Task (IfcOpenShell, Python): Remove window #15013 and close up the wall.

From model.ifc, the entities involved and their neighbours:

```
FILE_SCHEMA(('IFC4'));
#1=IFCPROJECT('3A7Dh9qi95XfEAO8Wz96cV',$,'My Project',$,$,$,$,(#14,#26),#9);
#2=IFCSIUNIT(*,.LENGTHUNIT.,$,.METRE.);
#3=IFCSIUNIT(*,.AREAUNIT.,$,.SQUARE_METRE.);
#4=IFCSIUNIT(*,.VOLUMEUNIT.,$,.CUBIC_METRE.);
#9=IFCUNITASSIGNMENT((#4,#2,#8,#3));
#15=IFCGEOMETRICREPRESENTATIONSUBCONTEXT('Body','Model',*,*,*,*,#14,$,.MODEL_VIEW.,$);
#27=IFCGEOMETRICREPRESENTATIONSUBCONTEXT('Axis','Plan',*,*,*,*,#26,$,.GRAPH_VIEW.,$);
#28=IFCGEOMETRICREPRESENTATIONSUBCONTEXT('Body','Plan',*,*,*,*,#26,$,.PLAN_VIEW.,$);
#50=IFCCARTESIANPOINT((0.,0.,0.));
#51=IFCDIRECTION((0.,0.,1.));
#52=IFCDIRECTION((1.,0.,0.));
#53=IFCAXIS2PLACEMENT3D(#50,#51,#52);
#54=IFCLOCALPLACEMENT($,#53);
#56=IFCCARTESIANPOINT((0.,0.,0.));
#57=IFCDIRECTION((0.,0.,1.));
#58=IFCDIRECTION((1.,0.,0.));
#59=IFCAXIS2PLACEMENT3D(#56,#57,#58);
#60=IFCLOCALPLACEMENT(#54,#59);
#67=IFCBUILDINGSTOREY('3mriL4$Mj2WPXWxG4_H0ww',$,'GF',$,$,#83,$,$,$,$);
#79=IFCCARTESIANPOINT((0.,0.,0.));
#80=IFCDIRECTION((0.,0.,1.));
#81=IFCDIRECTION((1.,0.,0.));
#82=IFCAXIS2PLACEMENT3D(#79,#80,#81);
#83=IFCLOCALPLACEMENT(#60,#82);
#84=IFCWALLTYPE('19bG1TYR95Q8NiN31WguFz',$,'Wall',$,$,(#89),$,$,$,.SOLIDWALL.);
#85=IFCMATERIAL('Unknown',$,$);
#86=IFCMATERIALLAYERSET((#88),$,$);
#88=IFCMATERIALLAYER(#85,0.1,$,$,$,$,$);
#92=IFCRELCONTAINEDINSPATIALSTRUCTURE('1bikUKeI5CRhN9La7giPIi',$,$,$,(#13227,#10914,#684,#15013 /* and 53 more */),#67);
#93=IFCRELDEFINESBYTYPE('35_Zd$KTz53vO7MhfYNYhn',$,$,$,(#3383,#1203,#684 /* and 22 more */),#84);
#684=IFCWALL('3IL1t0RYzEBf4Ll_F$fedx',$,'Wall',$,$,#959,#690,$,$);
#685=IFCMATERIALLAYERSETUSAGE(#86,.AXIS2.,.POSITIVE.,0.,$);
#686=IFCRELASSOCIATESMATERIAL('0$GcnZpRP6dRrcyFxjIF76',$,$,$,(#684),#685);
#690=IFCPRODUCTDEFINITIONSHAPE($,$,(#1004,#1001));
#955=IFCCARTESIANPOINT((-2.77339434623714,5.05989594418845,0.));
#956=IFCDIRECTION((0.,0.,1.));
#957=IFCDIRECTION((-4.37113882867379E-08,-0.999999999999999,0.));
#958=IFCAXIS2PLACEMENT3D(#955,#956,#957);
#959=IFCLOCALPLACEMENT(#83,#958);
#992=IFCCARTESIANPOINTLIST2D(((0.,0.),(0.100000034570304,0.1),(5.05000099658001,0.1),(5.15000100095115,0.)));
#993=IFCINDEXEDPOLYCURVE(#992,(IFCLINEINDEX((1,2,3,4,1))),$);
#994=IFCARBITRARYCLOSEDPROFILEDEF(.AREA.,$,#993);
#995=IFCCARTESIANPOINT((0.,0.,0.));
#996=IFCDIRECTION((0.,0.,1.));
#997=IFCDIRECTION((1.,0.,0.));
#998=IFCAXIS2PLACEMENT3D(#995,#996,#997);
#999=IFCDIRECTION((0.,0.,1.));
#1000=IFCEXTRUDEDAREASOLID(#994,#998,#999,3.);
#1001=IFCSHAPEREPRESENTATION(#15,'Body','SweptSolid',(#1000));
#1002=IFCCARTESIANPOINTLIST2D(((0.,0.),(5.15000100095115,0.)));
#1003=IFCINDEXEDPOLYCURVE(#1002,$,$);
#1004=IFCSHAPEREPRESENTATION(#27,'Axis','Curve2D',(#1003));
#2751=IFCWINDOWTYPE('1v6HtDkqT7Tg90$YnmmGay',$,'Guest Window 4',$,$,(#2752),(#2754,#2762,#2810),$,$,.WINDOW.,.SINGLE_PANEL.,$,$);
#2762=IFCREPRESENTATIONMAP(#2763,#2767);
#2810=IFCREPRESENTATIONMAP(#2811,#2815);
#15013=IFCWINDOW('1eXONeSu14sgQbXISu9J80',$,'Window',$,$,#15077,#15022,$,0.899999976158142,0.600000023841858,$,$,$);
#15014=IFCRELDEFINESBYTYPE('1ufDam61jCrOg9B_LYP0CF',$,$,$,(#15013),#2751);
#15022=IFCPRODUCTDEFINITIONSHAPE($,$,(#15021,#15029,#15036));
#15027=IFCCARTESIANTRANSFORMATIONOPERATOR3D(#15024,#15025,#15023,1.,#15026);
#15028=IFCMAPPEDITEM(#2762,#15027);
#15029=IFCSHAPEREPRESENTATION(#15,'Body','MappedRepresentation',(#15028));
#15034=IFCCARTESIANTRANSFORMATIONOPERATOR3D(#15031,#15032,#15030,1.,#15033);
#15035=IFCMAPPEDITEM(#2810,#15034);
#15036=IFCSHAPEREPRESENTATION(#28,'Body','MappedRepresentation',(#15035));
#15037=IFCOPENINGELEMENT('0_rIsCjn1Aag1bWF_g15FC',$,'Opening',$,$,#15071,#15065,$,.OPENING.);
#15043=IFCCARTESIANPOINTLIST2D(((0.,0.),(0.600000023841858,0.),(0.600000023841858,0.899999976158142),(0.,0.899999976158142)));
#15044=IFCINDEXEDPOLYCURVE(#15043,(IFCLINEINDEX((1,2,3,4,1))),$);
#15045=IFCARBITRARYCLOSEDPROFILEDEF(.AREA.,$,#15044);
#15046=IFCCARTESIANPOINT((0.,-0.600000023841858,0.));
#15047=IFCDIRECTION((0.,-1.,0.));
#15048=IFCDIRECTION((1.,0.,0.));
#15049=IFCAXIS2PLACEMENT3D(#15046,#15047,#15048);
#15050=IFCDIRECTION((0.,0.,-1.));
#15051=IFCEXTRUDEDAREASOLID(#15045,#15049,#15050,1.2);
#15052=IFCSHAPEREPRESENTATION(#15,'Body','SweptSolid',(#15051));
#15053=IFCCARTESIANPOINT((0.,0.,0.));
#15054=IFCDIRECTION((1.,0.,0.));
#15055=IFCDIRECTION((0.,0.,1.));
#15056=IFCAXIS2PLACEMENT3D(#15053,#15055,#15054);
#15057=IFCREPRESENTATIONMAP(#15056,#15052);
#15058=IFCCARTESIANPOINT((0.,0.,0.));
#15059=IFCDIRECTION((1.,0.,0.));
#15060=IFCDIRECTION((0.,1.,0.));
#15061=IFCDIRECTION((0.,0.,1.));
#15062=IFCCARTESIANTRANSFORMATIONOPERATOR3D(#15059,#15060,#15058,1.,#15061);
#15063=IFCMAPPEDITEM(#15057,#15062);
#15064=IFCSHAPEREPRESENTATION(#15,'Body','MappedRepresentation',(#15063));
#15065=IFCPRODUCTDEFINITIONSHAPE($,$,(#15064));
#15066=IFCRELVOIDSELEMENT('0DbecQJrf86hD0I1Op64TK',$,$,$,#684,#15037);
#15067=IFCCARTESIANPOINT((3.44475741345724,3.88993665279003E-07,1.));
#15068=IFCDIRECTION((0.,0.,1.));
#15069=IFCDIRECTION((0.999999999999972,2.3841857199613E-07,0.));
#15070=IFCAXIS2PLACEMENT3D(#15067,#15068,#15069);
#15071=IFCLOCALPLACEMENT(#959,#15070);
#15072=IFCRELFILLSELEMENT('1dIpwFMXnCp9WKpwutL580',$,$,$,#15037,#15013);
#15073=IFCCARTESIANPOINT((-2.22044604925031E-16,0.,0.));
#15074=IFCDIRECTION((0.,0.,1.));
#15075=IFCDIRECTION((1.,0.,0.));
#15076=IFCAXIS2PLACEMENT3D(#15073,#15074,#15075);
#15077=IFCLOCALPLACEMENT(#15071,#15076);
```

```python
import ifcopenshell
import ifcopenshell.api.feature
import ifcopenshell.api.root
import ifcopenshell.geom
import ifcopenshell.util.shape

model = ifcopenshell.open("model.ifc")
settings = ifcopenshell.geom.settings()


def volume(element):
    """Net volume in cubic metres, openings subtracted."""
    shape = ifcopenshell.geom.create_shape(settings, element)
    return ifcopenshell.util.shape.get_volume(shape.geometry)


window = model.by_guid("1eXONeSu14sgQbXISu9J80")
opening = window.FillsVoids[0].RelatingOpeningElement
wall = opening.VoidsElements[0].RelatingBuildingElement
before = volume(wall)

ifcopenshell.api.root.remove_product(model, product=window)
ifcopenshell.api.feature.remove_feature(model, feature=opening)

after = volume(wall)

print(f"wall volume {before:.3f} -> {after:.3f} m3")

model.write("model-out.ifc")
```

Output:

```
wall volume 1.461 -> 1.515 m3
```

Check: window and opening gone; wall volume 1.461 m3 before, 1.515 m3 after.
